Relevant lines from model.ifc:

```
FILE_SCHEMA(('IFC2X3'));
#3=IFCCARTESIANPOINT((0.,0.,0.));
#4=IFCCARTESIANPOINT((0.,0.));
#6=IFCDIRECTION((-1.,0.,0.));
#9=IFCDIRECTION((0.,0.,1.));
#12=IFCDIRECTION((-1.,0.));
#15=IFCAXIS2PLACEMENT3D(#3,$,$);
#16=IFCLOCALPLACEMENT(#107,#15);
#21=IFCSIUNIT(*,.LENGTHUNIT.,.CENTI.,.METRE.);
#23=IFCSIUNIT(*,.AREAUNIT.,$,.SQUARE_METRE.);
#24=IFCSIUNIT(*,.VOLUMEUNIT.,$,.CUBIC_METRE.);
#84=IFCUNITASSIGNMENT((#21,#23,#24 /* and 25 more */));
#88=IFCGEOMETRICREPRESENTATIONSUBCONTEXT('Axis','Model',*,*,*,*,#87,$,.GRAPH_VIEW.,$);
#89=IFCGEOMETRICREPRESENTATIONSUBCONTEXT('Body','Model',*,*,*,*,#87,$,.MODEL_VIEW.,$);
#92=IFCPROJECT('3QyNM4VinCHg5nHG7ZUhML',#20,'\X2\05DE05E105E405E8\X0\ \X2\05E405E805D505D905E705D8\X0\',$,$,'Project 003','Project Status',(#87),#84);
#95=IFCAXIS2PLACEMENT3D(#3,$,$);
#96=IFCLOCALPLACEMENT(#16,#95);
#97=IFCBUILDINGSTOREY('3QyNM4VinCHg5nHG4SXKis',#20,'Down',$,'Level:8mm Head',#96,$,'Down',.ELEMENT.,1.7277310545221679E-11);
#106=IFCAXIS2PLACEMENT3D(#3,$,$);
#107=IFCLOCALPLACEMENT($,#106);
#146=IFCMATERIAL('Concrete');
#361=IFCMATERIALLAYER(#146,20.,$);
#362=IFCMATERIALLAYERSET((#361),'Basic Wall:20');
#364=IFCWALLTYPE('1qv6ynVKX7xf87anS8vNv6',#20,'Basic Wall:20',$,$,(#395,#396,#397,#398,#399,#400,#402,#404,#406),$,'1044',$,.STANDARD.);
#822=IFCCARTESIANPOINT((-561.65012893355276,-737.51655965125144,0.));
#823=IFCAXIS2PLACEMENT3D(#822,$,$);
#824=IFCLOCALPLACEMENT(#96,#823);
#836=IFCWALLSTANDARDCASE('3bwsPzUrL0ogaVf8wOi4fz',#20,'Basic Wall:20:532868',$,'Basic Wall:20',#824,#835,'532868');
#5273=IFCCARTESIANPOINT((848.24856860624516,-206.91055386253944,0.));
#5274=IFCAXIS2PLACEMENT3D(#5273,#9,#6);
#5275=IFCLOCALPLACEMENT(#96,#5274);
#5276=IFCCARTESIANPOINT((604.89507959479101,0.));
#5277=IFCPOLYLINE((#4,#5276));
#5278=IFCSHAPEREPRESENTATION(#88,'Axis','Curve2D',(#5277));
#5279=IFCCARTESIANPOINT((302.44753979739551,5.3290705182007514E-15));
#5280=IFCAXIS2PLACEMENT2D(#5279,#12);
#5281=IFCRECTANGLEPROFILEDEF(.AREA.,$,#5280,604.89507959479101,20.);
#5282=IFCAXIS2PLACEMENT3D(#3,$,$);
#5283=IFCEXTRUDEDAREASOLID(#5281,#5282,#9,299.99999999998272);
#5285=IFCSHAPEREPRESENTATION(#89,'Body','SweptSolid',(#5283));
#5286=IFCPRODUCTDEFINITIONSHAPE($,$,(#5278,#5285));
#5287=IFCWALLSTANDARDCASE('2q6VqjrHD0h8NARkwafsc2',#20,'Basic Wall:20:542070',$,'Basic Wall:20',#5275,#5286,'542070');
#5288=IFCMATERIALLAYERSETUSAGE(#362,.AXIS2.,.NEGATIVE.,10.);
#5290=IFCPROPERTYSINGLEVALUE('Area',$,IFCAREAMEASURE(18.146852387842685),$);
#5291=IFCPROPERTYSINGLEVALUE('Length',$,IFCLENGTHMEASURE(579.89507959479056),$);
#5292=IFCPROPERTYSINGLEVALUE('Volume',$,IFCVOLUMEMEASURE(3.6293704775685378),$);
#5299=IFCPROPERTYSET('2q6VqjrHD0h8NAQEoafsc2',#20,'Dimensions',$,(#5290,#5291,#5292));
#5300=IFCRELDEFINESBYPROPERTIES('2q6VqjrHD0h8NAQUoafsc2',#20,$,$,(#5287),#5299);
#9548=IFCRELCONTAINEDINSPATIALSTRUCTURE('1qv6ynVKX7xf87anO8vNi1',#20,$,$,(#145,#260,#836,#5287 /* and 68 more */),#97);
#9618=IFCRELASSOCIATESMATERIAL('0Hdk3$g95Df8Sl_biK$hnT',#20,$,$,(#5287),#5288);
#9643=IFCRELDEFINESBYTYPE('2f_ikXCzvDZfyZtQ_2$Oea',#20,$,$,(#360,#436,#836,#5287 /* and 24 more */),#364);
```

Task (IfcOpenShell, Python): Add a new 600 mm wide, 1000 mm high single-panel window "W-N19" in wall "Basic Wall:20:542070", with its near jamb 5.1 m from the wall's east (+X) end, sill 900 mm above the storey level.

```python
import numpy as np
import ifcopenshell
import ifcopenshell.api.feature
import ifcopenshell.api.geometry
import ifcopenshell.api.pset
import ifcopenshell.api.root
import ifcopenshell.api.spatial
import ifcopenshell.api.type
import ifcopenshell.geom
import ifcopenshell.util.element
import ifcopenshell.util.placement
import ifcopenshell.util.representation
import ifcopenshell.util.shape
import ifcopenshell.util.unit

model = ifcopenshell.open("model.ifc")
unit_scale = ifcopenshell.util.unit.calculate_unit_scale(model)
area_scale = ifcopenshell.util.unit.calculate_unit_scale(model, "AREAUNIT")
volume_scale = ifcopenshell.util.unit.calculate_unit_scale(model, "VOLUMEUNIT")
settings = ifcopenshell.geom.settings()


def volume(element):
    """Net volume in cubic metres, openings subtracted."""
    shape = ifcopenshell.geom.create_shape(settings, element)
    return ifcopenshell.util.shape.get_volume(shape.geometry)


wall = model.by_id(5287)
storey = ifcopenshell.util.element.get_container(wall, ifc_class="IfcBuildingStorey")
context = ifcopenshell.util.representation.get_context(model, "Model", "Body", "MODEL_VIEW")
before = volume(wall)

width, height, from_end, sill = 0.6, 1, 5.1, 0.9  # metres

# The wall runs along its own X axis, and the end named is its -X end.
wall_shape = ifcopenshell.geom.create_shape(settings, wall)
x, y, z = ifcopenshell.util.shape.get_vertices(wall_shape.geometry).T
start = x.min() + from_end
face, thickness = float(y.min()), float(y.max() - y.min())
wall_matrix = ifcopenshell.util.placement.get_local_placement(wall.ObjectPlacement)
level = ifcopenshell.util.placement.get_local_placement(storey.ObjectPlacement)[2, 3]


def in_wall(x, y):
    """Placement at x, y metres in the wall's axes, at sill height."""
    matrix = wall_matrix.copy()
    matrix[:, 3] = wall_matrix @ np.array([x / unit_scale, y / unit_scale, 0.0, 1.0])
    matrix[2, 3] = level + sill / unit_scale
    return matrix


# Opening: a box that overshoots both wall faces by 50 mm.
opening = ifcopenshell.api.root.create_entity(model, ifc_class="IfcOpeningElement")
box = ifcopenshell.api.geometry.add_wall_representation(
    model, context=context, length=width, height=height, thickness=thickness + 0.1
)
ifcopenshell.api.geometry.assign_representation(model, product=opening, representation=box)
ifcopenshell.api.geometry.edit_object_placement(model, product=opening, matrix=in_wall(start, face - 0.05), is_si=False)
ifcopenshell.api.feature.add_feature(model, feature=opening, element=wall)

window = ifcopenshell.api.root.create_entity(model, ifc_class="IfcWindow", name="W-N19")
window.OverallWidth, window.OverallHeight = width / unit_scale, height / unit_scale
body = ifcopenshell.api.geometry.add_window_representation(
    model,
    context=context,
    overall_width=window.OverallWidth,
    overall_height=window.OverallHeight,
    partition_type="SINGLE_PANEL",
)
ifcopenshell.api.geometry.assign_representation(model, product=window, representation=body)
ifcopenshell.api.spatial.assign_container(model, products=[window], relating_structure=storey)
fills = ifcopenshell.api.feature.add_filling(model, opening=opening, element=window)
fills.OwnerHistory = window.OwnerHistory  # required in IFC2X3

# IFC2X3 keeps the operation on the window style.
style = ifcopenshell.api.root.create_entity(model, ifc_class="IfcWindowStyle", name="W-N19")
style.OperationType, style.ConstructionType = "SINGLE_PANEL", "NOTDEFINED"
style.ParameterTakesPrecedence = style.Sizeable = False
ifcopenshell.api.type.assign_type(model, related_objects=[window], relating_type=style)

# Centre the window in the wall's thickness.
ifcopenshell.api.geometry.edit_object_placement(model, product=window, matrix=in_wall(start, face), is_si=False)
window_shape = ifcopenshell.geom.create_shape(settings, window)
depth = ifcopenshell.util.shape.get_vertices(window_shape.geometry)[:, 1]
offset = face + thickness / 2 - (depth.min() + depth.max()) / 2
ifcopenshell.api.geometry.edit_object_placement(model, product=window, matrix=in_wall(start, offset), is_si=False)

after = volume(wall)

# Update the wall's stored quantities.
pset = model.by_id(ifcopenshell.util.element.get_pset(wall, "Dimensions", should_inherit=False)["id"])
ifcopenshell.api.pset.edit_pset(model, pset=pset, properties={
    "Area": model.create_entity("IfcAreaMeasure", after / thickness / area_scale),
    "Volume": model.create_entity("IfcVolumeMeasure", after / volume_scale),
})

print(f"wall volume {before:.3f} -> {after:.3f} m3")

model.write("model_updated.ifc")
```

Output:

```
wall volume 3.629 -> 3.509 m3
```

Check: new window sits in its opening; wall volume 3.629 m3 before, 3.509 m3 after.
